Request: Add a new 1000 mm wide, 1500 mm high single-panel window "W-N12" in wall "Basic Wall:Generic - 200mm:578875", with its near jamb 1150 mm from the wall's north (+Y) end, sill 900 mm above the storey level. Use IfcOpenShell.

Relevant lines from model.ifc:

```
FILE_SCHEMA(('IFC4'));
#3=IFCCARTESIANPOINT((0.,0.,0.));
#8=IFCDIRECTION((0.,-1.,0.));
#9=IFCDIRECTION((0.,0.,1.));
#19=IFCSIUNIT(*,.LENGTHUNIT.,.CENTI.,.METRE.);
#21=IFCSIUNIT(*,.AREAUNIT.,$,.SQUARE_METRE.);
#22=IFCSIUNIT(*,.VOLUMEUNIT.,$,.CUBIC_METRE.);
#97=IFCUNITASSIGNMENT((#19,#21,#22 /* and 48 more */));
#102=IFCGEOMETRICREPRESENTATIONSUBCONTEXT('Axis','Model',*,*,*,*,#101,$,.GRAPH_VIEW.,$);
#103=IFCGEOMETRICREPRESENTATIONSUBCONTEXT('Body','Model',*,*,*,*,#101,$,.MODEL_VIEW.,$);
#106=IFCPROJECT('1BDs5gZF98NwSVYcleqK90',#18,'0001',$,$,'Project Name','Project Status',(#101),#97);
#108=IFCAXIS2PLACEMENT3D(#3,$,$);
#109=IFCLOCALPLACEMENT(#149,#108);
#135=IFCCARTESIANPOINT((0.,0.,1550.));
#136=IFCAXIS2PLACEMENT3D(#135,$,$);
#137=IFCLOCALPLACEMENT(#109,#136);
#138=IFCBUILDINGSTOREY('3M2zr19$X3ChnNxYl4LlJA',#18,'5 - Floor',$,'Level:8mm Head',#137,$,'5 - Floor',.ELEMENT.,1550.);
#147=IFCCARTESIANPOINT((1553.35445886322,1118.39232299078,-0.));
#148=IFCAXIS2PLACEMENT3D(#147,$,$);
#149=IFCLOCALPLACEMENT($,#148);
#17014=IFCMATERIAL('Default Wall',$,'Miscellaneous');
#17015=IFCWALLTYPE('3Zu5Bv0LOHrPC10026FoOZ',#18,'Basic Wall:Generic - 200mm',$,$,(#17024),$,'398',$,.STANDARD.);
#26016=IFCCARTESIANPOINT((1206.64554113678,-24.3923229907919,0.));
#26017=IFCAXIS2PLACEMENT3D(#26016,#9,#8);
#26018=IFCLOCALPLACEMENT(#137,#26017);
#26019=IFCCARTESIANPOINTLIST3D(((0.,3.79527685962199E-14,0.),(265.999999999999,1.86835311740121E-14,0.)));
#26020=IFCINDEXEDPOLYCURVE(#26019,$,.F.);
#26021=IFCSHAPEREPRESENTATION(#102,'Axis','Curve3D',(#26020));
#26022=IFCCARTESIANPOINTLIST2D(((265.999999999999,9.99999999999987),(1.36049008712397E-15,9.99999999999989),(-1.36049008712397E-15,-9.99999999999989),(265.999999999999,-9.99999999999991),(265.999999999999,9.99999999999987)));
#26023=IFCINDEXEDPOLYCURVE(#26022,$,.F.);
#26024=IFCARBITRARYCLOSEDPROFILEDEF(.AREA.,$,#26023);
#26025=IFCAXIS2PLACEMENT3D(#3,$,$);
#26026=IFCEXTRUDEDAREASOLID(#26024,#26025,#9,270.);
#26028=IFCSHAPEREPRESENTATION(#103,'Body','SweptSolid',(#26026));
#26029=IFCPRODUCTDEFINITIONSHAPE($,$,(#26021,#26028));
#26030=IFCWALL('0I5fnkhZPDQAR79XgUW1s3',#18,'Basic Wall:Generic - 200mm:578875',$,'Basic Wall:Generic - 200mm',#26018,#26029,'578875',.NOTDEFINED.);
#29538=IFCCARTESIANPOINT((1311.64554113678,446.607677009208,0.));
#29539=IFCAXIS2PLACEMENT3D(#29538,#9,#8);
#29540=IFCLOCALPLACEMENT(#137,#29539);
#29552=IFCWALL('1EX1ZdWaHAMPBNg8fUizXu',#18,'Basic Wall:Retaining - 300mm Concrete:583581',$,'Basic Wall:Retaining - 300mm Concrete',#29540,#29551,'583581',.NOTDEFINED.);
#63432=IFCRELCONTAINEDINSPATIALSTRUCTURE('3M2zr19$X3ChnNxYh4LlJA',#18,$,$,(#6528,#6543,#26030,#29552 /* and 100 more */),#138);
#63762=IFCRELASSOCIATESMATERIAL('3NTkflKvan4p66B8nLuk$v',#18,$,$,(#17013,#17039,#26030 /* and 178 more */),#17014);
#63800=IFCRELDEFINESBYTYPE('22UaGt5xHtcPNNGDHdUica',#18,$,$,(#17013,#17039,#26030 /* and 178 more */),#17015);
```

```python
import numpy as np
import ifcopenshell
import ifcopenshell.api.feature
import ifcopenshell.api.geometry
import ifcopenshell.api.root
import ifcopenshell.api.spatial
import ifcopenshell.geom
import ifcopenshell.util.element
import ifcopenshell.util.placement
import ifcopenshell.util.representation
import ifcopenshell.util.shape
import ifcopenshell.util.unit

model = ifcopenshell.open("model.ifc")
unit_scale = ifcopenshell.util.unit.calculate_unit_scale(model)
settings = ifcopenshell.geom.settings()


def volume(element):
    """Net volume in cubic metres, openings subtracted."""
    shape = ifcopenshell.geom.create_shape(settings, element)
    return ifcopenshell.util.shape.get_volume(shape.geometry)


wall = model.by_id(26030)
storey = ifcopenshell.util.element.get_container(wall, ifc_class="IfcBuildingStorey")
context = ifcopenshell.util.representation.get_context(model, "Model", "Body", "MODEL_VIEW")
before = volume(wall)

width, height, from_end, sill = 1, 1.5, 1.15, 0.9  # metres

# The wall runs along its own X axis, and the end named is its -X end.
wall_shape = ifcopenshell.geom.create_shape(settings, wall)
x, y, z = ifcopenshell.util.shape.get_vertices(wall_shape.geometry).T
start = x.min() + from_end
face, thickness = float(y.min()), float(y.max() - y.min())
wall_matrix = ifcopenshell.util.placement.get_local_placement(wall.ObjectPlacement)
level = ifcopenshell.util.placement.get_local_placement(storey.ObjectPlacement)[2, 3]


def in_wall(x, y):
    """Placement at x, y metres in the wall's axes, at sill height."""
    matrix = wall_matrix.copy()
    matrix[:, 3] = wall_matrix @ np.array([x / unit_scale, y / unit_scale, 0.0, 1.0])
    matrix[2, 3] = level + sill / unit_scale
    return matrix


# Opening: a box that overshoots both wall faces by 50 mm.
opening = ifcopenshell.api.root.create_entity(model, ifc_class="IfcOpeningElement", predefined_type="OPENING")
box = ifcopenshell.api.geometry.add_wall_representation(
    model, context=context, length=width, height=height, thickness=thickness + 0.1
)
ifcopenshell.api.geometry.assign_representation(model, product=opening, representation=box)
ifcopenshell.api.geometry.edit_object_placement(model, product=opening, matrix=in_wall(start, face - 0.05), is_si=False)
ifcopenshell.api.feature.add_feature(model, feature=opening, element=wall)

window = ifcopenshell.api.root.create_entity(model, ifc_class="IfcWindow", name="W-N12", predefined_type="WINDOW")
window.OverallWidth, window.OverallHeight = width / unit_scale, height / unit_scale
window.PartitioningType = "SINGLE_PANEL"
body = ifcopenshell.api.geometry.add_window_representation(
    model,
    context=context,
    overall_width=window.OverallWidth,
    overall_height=window.OverallHeight,
    partition_type="SINGLE_PANEL",
)
ifcopenshell.api.geometry.assign_representation(model, product=window, representation=body)
ifcopenshell.api.spatial.assign_container(model, products=[window], relating_structure=storey)
ifcopenshell.api.feature.add_filling(model, opening=opening, element=window)

# Centre the window in the wall's thickness.
ifcopenshell.api.geometry.edit_object_placement(model, product=window, matrix=in_wall(start, face), is_si=False)
window_shape = ifcopenshell.geom.create_shape(settings, window)
depth = ifcopenshell.util.shape.get_vertices(window_shape.geometry)[:, 1]
offset = face + thickness / 2 - (depth.min() + depth.max()) / 2
ifcopenshell.api.geometry.edit_object_placement(model, product=window, matrix=in_wall(start, offset), is_si=False)

after = volume(wall)

print(f"wall volume {before:.3f} -> {after:.3f} m3")

model.write("model_v2.ifc")
```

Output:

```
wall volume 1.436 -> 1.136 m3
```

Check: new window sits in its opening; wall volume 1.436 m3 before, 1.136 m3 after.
